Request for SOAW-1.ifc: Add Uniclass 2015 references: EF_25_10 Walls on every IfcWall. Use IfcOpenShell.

First a look at what the model holds.

```python
import ifcopenshell

model = ifcopenshell.open("SOAW-1.ifc")
print(model.schema)
print("classifications:", [c.Name for c in model.by_type("IfcClassification")])
for ifc_class in ("IfcDoor", "IfcRoof", "IfcStair", "IfcWall", "IfcWindow"):
    print(ifc_class, len(model.by_type(ifc_class)))
```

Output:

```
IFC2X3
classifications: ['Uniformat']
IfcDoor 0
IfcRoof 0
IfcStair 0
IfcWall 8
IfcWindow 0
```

```python
import ifcopenshell
import ifcopenshell.api.classification

model = ifcopenshell.open("SOAW-1.ifc")

# IFC2X3 requires Source and Edition and has no link from the project to the system.
system = model.create_entity("IfcClassification", Source="NBS", Edition="2015", Name="Uniclass 2015")

codes = {
    "IfcWall": ("EF_25_10", "Walls"),
}
for ifc_class, (code, name) in codes.items():
    products = model.by_type(ifc_class)
    ifcopenshell.api.classification.add_reference(
        model, products=products, classification=system, identification=code, name=name
    )
    print(code, len(products))

model.write("SOAW-1-out.ifc")
```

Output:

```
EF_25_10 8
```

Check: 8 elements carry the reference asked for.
